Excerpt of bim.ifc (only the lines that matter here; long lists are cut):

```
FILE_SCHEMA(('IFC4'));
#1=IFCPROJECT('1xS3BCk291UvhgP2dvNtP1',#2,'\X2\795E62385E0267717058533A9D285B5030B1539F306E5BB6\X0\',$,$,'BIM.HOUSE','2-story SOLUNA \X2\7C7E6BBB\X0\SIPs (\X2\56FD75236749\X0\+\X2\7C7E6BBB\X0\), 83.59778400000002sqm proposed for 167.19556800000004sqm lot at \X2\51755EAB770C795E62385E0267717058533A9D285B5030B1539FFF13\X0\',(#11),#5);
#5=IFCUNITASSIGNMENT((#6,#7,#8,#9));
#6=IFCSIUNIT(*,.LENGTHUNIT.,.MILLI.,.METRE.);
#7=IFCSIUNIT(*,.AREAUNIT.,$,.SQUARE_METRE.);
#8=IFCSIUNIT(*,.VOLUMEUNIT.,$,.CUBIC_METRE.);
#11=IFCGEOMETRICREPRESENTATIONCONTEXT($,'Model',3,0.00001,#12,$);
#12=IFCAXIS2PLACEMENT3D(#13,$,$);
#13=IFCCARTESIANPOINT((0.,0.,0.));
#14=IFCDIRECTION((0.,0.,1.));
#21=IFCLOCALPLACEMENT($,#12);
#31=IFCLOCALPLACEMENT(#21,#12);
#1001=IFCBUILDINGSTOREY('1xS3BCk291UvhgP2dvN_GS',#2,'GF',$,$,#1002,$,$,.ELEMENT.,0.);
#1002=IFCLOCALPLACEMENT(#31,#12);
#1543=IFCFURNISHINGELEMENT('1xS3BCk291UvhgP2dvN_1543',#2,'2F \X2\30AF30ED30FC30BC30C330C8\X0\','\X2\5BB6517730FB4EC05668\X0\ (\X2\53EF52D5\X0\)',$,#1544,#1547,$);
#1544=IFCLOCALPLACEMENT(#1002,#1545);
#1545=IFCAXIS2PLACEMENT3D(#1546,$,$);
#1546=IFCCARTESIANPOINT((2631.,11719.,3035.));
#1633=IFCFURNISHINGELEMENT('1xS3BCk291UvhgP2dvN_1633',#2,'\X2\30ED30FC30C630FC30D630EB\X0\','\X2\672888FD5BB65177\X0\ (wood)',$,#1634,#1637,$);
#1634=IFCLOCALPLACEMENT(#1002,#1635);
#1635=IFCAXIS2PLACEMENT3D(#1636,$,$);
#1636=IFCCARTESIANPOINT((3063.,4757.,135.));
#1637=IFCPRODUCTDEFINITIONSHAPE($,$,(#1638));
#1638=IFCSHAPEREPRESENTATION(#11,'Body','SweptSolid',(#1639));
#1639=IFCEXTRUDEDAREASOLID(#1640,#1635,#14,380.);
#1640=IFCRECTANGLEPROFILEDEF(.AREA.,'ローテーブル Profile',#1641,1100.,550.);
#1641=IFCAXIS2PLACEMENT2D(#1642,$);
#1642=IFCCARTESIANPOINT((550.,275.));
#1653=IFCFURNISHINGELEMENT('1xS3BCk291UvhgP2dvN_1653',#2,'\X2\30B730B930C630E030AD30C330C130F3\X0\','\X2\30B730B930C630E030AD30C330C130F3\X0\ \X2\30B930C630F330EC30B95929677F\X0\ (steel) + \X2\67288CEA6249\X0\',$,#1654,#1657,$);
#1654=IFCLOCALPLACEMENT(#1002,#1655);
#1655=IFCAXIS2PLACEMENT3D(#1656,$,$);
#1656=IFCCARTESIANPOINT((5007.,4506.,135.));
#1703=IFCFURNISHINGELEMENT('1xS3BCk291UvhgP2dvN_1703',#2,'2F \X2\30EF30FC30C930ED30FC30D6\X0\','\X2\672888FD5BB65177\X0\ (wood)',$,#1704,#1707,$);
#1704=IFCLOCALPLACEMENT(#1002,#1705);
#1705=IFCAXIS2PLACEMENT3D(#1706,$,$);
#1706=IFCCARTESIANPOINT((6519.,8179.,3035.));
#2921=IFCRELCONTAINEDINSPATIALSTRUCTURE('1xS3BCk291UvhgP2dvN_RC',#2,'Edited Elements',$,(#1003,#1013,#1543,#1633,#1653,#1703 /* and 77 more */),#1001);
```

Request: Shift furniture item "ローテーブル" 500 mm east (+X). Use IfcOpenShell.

```python
import ifcopenshell
import ifcopenshell.api.geometry
import ifcopenshell.util.placement
import ifcopenshell.util.unit

model = ifcopenshell.open("bim.ifc")
unit_scale = ifcopenshell.util.unit.calculate_unit_scale(model)

item = model.by_guid("1xS3BCk291UvhgP2dvN_1633")
matrix = ifcopenshell.util.placement.get_local_placement(item.ObjectPlacement)
matrix[0, 3] += 0.5 / unit_scale
ifcopenshell.api.geometry.edit_object_placement(model, product=item, matrix=matrix, is_si=False)

print(ifcopenshell.util.placement.get_local_placement(item.ObjectPlacement).round(3) + 0.0)

model.write("bim_updated.ifc")
```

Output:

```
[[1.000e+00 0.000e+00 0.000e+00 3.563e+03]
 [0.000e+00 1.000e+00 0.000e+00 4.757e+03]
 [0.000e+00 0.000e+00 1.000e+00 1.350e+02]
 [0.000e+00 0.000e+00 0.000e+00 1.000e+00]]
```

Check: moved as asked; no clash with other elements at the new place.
